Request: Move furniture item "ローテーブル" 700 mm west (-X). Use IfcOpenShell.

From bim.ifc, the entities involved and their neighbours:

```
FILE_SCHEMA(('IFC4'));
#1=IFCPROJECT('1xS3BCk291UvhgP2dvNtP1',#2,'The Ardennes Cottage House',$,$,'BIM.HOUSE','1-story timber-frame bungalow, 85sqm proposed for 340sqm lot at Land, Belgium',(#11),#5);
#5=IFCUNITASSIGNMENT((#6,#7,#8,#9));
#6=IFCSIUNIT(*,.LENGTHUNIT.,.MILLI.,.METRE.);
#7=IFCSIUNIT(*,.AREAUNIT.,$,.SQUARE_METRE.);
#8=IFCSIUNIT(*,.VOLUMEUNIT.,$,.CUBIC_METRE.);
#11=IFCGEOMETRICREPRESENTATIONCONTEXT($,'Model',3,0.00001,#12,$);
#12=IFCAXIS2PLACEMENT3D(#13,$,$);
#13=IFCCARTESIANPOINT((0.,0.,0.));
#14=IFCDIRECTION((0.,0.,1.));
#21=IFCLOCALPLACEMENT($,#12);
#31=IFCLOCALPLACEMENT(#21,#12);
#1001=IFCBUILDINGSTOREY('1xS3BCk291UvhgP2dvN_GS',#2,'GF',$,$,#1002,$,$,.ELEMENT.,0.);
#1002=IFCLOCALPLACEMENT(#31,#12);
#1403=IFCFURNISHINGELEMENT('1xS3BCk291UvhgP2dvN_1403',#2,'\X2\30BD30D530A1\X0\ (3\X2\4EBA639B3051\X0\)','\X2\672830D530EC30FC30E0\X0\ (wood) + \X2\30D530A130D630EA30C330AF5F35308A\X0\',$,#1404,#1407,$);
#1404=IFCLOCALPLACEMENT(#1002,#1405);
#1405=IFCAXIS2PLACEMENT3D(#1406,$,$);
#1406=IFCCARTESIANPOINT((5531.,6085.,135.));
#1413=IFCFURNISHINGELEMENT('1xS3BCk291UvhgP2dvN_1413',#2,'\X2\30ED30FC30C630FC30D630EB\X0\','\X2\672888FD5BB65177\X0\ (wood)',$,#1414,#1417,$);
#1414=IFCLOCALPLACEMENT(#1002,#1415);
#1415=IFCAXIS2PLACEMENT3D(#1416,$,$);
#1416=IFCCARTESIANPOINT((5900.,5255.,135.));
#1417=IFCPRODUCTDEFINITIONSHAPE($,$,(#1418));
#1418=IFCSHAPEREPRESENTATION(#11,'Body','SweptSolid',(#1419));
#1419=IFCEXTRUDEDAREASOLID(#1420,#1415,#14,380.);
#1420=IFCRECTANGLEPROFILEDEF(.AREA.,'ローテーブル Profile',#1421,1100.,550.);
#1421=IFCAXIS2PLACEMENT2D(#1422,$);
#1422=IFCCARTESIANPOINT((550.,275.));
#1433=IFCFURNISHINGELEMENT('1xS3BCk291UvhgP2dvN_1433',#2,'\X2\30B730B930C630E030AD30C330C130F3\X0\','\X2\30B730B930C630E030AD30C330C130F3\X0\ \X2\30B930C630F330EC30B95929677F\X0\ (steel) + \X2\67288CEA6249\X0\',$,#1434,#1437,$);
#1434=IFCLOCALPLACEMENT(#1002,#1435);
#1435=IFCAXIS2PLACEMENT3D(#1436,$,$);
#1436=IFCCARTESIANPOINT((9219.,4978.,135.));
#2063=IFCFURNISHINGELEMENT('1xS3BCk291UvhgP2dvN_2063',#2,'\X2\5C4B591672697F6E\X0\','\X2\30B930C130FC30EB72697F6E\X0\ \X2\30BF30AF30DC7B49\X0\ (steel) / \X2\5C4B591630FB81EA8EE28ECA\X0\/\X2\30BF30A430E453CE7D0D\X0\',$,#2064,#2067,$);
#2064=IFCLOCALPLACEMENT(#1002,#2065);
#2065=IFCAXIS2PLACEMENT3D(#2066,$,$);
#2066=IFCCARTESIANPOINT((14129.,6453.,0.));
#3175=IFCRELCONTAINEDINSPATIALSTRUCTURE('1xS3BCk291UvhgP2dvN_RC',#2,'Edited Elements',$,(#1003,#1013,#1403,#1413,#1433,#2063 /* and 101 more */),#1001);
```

```python
import ifcopenshell
import ifcopenshell.api.geometry
import ifcopenshell.util.placement
import ifcopenshell.util.unit

model = ifcopenshell.open("bim.ifc")
unit_scale = ifcopenshell.util.unit.calculate_unit_scale(model)

item = model.by_id(1413)
matrix = ifcopenshell.util.placement.get_local_placement(item.ObjectPlacement)
matrix[0, 3] -= 0.7 / unit_scale
ifcopenshell.api.geometry.edit_object_placement(model, product=item, matrix=matrix, is_si=False)

print(ifcopenshell.util.placement.get_local_placement(item.ObjectPlacement).round(3) + 0.0)

model.write("bim_v2.ifc")
```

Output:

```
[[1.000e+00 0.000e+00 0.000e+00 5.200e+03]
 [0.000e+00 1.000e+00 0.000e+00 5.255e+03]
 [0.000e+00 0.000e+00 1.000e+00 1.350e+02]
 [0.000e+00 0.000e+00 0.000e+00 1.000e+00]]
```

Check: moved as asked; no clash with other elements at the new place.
